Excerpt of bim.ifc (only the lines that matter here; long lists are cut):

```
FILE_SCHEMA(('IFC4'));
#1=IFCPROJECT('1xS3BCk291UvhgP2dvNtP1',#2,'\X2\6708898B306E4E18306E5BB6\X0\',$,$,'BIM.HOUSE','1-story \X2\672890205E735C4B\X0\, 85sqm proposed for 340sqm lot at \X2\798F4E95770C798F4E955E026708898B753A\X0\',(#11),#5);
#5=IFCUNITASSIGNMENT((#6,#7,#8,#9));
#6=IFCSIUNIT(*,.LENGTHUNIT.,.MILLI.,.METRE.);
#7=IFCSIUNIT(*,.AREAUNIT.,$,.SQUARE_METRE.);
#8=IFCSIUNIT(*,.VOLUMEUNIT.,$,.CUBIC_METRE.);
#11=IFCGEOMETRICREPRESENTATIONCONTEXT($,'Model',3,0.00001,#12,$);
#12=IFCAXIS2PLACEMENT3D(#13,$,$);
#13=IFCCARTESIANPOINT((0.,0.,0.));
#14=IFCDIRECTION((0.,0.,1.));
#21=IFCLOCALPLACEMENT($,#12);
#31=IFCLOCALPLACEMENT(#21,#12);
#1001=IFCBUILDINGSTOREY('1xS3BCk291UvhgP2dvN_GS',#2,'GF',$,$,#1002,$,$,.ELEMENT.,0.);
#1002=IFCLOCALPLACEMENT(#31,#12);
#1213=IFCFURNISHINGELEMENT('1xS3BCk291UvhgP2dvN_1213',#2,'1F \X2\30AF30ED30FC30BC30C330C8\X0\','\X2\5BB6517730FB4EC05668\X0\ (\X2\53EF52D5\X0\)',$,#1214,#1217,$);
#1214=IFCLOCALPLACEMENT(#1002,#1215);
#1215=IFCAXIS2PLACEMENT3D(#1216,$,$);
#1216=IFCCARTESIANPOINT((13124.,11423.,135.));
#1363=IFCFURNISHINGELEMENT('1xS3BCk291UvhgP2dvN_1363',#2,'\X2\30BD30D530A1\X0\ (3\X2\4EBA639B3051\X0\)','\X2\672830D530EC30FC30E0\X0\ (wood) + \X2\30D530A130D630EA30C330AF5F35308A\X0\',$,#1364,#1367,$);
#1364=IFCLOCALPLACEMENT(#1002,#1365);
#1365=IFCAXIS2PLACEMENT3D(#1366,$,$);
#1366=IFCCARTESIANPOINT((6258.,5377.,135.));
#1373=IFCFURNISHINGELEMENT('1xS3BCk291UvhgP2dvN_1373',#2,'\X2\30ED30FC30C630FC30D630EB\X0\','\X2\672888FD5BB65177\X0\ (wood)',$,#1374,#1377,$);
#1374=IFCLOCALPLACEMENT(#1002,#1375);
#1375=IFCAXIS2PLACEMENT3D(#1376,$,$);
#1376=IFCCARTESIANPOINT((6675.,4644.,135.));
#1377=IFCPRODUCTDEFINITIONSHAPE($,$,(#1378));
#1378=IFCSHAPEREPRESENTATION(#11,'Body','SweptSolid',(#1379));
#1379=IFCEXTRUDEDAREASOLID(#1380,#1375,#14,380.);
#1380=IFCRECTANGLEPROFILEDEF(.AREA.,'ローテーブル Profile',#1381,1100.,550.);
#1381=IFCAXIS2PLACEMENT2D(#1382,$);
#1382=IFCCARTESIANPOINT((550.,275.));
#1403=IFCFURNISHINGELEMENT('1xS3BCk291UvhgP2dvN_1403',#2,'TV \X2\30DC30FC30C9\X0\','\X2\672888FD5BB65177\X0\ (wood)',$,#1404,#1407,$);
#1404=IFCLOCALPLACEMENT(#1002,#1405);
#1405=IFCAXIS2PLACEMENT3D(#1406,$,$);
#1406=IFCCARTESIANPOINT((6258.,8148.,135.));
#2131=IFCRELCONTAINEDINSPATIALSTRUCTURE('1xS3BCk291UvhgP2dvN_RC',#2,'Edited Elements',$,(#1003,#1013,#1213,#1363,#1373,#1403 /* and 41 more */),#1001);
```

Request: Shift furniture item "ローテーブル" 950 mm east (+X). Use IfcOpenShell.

```python
import ifcopenshell
import ifcopenshell.api.geometry
import ifcopenshell.util.placement
import ifcopenshell.util.unit

model = ifcopenshell.open("bim.ifc")
unit_scale = ifcopenshell.util.unit.calculate_unit_scale(model)

item = model.by_guid("1xS3BCk291UvhgP2dvN_1373")
matrix = ifcopenshell.util.placement.get_local_placement(item.ObjectPlacement)
matrix[0, 3] += 0.95 / unit_scale
ifcopenshell.api.geometry.edit_object_placement(model, product=item, matrix=matrix, is_si=False)

print(ifcopenshell.util.placement.get_local_placement(item.ObjectPlacement).round(3) + 0.0)

model.write("bim_edited.ifc")
```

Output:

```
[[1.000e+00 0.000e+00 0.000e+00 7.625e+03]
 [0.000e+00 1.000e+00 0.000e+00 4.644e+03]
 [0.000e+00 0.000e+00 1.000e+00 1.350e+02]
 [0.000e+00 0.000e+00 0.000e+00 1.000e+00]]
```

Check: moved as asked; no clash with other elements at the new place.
